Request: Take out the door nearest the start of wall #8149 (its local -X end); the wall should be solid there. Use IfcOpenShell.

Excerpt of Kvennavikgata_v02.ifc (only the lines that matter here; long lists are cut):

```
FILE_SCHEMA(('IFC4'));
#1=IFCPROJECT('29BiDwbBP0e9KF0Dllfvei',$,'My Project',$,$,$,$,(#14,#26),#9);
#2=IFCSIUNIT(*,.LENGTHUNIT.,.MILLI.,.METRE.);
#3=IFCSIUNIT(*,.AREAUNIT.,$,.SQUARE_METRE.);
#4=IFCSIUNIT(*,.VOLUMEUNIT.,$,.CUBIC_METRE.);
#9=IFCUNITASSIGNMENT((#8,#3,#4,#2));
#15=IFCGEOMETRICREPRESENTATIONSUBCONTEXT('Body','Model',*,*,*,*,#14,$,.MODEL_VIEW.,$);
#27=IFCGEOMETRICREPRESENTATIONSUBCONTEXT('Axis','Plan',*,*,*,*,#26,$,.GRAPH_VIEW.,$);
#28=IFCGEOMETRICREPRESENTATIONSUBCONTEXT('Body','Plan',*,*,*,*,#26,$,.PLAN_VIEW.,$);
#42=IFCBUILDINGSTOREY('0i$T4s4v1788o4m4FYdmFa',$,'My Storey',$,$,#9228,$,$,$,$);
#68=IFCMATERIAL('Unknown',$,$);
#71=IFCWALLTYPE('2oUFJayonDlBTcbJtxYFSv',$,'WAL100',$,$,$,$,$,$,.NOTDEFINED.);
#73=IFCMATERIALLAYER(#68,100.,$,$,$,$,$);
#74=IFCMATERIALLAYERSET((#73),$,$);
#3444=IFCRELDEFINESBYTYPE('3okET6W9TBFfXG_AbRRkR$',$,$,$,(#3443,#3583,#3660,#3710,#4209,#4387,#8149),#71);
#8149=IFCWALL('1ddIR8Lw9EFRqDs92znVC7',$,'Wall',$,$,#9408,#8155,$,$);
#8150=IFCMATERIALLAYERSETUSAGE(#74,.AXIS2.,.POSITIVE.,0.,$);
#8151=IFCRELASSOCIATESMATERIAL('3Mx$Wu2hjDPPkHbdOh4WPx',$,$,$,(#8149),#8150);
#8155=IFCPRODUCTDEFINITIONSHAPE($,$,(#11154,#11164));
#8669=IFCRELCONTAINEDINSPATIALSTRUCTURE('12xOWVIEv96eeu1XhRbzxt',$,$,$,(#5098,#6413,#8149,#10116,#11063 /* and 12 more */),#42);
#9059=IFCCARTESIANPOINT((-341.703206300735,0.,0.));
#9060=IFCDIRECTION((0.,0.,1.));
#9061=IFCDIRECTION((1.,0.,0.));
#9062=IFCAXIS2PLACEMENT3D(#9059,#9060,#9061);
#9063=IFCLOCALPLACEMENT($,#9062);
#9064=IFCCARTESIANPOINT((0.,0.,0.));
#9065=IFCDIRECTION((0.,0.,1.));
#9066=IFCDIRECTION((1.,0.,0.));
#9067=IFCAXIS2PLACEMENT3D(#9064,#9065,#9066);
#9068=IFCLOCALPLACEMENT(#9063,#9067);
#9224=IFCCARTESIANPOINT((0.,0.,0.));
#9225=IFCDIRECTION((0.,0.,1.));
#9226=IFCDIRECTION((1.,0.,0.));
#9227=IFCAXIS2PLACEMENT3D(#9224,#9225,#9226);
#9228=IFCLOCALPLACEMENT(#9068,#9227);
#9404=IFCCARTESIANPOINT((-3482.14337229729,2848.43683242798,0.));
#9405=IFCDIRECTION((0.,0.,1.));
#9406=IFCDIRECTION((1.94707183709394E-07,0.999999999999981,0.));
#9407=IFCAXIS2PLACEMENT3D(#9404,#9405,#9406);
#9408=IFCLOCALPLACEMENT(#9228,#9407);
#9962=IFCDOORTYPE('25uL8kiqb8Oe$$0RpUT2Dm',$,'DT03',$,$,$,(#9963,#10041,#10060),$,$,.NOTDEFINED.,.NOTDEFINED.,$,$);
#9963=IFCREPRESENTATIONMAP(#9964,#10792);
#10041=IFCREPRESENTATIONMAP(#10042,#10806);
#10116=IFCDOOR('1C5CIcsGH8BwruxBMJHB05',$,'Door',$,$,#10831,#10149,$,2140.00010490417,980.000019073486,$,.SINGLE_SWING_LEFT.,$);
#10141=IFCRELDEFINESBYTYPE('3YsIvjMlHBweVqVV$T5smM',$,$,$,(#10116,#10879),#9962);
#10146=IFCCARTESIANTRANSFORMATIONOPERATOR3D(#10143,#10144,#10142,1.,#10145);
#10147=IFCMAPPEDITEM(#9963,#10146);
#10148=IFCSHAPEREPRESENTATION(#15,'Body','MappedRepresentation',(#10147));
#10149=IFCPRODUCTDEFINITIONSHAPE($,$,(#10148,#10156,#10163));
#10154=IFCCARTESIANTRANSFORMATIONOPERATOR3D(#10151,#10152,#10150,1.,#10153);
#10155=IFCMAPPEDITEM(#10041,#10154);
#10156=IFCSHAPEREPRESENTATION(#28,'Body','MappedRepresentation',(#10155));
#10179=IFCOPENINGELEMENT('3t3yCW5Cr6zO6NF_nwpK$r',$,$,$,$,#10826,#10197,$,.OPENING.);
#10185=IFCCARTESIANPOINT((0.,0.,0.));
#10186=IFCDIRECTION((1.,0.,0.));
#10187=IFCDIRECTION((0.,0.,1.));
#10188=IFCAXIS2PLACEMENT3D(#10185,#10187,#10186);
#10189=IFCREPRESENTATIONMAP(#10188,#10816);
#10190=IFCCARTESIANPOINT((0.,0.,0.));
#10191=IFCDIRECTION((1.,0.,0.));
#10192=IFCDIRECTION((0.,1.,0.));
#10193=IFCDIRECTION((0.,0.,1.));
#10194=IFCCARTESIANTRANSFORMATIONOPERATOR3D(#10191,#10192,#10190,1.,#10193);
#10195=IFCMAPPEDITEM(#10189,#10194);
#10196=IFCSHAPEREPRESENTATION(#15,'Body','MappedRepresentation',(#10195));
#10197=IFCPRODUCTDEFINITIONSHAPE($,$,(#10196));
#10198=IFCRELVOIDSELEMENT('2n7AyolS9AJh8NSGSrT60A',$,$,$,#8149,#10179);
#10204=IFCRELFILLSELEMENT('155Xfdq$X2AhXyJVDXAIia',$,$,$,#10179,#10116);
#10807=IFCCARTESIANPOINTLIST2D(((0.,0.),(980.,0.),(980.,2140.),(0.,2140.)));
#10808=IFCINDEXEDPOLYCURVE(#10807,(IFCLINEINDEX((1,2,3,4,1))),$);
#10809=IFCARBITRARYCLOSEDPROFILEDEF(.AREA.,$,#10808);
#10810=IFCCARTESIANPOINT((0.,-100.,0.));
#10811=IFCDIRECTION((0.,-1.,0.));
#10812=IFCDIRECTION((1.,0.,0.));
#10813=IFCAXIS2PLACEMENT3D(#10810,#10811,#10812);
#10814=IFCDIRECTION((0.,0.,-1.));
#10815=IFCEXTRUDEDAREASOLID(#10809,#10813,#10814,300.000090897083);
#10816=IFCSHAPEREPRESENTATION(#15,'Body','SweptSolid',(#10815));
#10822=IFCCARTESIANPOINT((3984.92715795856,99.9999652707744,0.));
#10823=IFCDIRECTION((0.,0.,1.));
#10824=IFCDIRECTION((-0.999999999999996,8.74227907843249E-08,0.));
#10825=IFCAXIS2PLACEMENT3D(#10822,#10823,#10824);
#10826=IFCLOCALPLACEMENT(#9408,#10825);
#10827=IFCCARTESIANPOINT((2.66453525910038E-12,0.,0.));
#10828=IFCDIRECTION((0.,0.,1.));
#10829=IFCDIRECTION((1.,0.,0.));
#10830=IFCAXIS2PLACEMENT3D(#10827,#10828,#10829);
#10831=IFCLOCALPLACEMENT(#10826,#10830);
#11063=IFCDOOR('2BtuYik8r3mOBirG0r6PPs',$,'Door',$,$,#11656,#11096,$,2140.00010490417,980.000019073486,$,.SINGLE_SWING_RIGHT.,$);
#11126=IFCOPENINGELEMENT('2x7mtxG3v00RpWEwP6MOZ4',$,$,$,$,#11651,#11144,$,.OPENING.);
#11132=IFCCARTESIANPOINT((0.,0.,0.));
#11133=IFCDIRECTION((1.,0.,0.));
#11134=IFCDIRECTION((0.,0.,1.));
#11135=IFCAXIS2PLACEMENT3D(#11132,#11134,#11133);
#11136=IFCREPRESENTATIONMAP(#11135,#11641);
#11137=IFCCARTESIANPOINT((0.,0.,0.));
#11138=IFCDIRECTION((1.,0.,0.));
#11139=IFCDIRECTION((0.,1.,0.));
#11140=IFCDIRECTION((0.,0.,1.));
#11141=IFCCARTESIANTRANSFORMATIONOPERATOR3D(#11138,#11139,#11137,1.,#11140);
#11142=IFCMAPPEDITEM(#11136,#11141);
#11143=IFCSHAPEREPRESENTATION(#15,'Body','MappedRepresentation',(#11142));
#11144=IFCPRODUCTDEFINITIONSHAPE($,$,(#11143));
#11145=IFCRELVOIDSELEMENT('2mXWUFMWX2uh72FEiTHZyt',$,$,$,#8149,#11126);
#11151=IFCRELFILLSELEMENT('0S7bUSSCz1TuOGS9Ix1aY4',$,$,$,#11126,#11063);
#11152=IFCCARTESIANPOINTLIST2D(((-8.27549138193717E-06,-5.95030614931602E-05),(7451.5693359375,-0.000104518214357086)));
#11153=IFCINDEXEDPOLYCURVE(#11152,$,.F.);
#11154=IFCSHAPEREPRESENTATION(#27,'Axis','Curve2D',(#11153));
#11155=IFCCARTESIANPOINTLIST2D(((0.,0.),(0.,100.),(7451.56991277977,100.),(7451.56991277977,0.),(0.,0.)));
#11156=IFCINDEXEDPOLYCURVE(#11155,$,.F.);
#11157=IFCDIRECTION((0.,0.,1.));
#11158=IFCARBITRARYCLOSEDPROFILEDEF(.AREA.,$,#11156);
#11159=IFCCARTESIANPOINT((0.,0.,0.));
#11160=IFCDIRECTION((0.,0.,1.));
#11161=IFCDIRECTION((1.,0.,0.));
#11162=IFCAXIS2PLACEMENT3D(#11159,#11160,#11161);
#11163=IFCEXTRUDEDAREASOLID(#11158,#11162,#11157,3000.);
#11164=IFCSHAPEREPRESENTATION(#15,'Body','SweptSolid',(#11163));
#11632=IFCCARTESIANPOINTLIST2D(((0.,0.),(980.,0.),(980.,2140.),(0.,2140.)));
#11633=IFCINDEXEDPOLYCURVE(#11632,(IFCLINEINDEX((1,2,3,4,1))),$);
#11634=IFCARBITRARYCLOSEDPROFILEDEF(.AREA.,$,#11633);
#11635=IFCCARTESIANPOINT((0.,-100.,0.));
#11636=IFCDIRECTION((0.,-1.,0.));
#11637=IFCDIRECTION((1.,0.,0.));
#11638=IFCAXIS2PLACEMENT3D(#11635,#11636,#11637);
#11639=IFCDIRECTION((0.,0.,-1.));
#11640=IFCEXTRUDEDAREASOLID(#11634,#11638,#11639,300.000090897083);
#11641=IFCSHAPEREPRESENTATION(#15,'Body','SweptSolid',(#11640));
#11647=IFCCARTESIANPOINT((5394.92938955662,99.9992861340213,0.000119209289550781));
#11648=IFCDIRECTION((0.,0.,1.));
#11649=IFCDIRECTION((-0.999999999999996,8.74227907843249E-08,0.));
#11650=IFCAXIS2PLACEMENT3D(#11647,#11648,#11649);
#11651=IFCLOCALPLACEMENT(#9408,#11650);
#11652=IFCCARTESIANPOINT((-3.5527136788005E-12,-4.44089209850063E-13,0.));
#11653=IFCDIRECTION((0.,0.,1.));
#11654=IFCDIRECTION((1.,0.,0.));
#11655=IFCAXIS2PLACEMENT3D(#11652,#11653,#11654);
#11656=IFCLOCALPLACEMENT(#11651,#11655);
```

```python
import ifcopenshell
import ifcopenshell.api.feature
import ifcopenshell.api.root
import ifcopenshell.geom
import ifcopenshell.util.shape

model = ifcopenshell.open("Kvennavikgata_v02.ifc")
settings = ifcopenshell.geom.settings()


def volume(element):
    """Net volume in cubic metres, openings subtracted."""
    shape = ifcopenshell.geom.create_shape(settings, element)
    return ifcopenshell.util.shape.get_volume(shape.geometry)


door = model.by_id(10116)
opening = door.FillsVoids[0].RelatingOpeningElement
wall = opening.VoidsElements[0].RelatingBuildingElement
before = volume(wall)

ifcopenshell.api.root.remove_product(model, product=door)
ifcopenshell.api.feature.remove_feature(model, feature=opening)

after = volume(wall)

print(f"wall volume {before:.3f} -> {after:.3f} m3")

model.write("Kvennavikgata_v02_v2.ifc")
```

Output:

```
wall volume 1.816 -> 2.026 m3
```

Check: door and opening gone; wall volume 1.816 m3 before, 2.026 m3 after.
